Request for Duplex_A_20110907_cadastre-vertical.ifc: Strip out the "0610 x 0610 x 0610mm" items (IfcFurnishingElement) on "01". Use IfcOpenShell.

First a look at what the model holds.

```python
import ifcopenshell
import ifcopenshell.util.element

model = ifcopenshell.open("Duplex_A_20110907_cadastre-vertical.ifc")
print(model.schema)
storey = next(s for s in model.by_type("IfcBuildingStorey") if s.Name == "01")
furniture = [e for e in ifcopenshell.util.element.get_decomposition(storey) if e.is_a("IfcFurnishingElement")]
seen = {}
for e in furniture:
    element_type = ifcopenshell.util.element.get_type(e)
    name = element_type.Name if element_type not in (None, e) else None
    seen[name] = seen.get(name, 0) + 1
for name, count in sorted(seen.items(), key=str):
    print(count, "x", name)
```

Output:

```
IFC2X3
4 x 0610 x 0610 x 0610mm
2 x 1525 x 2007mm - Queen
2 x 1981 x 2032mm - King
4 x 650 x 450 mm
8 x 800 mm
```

```python
import ifcopenshell
import ifcopenshell.api.root
import ifcopenshell.util.element

model = ifcopenshell.open("Duplex_A_20110907_cadastre-vertical.ifc")

storey = next(s for s in model.by_type("IfcBuildingStorey") if s.Name == "01")
furniture = [e for e in ifcopenshell.util.element.get_decomposition(storey) if e.is_a("IfcFurnishingElement")]
targets = [e for e in furniture if (t := ifcopenshell.util.element.get_type(e)) not in (None, e) and t.Name == "0610 x 0610 x 0610mm"]

for e in targets:
    ifcopenshell.api.root.remove_product(model, product=e)
print(len(targets), "removed")

model.write("Duplex_A_20110907_cadastre-vertical_edited.ifc")
```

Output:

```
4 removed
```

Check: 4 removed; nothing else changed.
